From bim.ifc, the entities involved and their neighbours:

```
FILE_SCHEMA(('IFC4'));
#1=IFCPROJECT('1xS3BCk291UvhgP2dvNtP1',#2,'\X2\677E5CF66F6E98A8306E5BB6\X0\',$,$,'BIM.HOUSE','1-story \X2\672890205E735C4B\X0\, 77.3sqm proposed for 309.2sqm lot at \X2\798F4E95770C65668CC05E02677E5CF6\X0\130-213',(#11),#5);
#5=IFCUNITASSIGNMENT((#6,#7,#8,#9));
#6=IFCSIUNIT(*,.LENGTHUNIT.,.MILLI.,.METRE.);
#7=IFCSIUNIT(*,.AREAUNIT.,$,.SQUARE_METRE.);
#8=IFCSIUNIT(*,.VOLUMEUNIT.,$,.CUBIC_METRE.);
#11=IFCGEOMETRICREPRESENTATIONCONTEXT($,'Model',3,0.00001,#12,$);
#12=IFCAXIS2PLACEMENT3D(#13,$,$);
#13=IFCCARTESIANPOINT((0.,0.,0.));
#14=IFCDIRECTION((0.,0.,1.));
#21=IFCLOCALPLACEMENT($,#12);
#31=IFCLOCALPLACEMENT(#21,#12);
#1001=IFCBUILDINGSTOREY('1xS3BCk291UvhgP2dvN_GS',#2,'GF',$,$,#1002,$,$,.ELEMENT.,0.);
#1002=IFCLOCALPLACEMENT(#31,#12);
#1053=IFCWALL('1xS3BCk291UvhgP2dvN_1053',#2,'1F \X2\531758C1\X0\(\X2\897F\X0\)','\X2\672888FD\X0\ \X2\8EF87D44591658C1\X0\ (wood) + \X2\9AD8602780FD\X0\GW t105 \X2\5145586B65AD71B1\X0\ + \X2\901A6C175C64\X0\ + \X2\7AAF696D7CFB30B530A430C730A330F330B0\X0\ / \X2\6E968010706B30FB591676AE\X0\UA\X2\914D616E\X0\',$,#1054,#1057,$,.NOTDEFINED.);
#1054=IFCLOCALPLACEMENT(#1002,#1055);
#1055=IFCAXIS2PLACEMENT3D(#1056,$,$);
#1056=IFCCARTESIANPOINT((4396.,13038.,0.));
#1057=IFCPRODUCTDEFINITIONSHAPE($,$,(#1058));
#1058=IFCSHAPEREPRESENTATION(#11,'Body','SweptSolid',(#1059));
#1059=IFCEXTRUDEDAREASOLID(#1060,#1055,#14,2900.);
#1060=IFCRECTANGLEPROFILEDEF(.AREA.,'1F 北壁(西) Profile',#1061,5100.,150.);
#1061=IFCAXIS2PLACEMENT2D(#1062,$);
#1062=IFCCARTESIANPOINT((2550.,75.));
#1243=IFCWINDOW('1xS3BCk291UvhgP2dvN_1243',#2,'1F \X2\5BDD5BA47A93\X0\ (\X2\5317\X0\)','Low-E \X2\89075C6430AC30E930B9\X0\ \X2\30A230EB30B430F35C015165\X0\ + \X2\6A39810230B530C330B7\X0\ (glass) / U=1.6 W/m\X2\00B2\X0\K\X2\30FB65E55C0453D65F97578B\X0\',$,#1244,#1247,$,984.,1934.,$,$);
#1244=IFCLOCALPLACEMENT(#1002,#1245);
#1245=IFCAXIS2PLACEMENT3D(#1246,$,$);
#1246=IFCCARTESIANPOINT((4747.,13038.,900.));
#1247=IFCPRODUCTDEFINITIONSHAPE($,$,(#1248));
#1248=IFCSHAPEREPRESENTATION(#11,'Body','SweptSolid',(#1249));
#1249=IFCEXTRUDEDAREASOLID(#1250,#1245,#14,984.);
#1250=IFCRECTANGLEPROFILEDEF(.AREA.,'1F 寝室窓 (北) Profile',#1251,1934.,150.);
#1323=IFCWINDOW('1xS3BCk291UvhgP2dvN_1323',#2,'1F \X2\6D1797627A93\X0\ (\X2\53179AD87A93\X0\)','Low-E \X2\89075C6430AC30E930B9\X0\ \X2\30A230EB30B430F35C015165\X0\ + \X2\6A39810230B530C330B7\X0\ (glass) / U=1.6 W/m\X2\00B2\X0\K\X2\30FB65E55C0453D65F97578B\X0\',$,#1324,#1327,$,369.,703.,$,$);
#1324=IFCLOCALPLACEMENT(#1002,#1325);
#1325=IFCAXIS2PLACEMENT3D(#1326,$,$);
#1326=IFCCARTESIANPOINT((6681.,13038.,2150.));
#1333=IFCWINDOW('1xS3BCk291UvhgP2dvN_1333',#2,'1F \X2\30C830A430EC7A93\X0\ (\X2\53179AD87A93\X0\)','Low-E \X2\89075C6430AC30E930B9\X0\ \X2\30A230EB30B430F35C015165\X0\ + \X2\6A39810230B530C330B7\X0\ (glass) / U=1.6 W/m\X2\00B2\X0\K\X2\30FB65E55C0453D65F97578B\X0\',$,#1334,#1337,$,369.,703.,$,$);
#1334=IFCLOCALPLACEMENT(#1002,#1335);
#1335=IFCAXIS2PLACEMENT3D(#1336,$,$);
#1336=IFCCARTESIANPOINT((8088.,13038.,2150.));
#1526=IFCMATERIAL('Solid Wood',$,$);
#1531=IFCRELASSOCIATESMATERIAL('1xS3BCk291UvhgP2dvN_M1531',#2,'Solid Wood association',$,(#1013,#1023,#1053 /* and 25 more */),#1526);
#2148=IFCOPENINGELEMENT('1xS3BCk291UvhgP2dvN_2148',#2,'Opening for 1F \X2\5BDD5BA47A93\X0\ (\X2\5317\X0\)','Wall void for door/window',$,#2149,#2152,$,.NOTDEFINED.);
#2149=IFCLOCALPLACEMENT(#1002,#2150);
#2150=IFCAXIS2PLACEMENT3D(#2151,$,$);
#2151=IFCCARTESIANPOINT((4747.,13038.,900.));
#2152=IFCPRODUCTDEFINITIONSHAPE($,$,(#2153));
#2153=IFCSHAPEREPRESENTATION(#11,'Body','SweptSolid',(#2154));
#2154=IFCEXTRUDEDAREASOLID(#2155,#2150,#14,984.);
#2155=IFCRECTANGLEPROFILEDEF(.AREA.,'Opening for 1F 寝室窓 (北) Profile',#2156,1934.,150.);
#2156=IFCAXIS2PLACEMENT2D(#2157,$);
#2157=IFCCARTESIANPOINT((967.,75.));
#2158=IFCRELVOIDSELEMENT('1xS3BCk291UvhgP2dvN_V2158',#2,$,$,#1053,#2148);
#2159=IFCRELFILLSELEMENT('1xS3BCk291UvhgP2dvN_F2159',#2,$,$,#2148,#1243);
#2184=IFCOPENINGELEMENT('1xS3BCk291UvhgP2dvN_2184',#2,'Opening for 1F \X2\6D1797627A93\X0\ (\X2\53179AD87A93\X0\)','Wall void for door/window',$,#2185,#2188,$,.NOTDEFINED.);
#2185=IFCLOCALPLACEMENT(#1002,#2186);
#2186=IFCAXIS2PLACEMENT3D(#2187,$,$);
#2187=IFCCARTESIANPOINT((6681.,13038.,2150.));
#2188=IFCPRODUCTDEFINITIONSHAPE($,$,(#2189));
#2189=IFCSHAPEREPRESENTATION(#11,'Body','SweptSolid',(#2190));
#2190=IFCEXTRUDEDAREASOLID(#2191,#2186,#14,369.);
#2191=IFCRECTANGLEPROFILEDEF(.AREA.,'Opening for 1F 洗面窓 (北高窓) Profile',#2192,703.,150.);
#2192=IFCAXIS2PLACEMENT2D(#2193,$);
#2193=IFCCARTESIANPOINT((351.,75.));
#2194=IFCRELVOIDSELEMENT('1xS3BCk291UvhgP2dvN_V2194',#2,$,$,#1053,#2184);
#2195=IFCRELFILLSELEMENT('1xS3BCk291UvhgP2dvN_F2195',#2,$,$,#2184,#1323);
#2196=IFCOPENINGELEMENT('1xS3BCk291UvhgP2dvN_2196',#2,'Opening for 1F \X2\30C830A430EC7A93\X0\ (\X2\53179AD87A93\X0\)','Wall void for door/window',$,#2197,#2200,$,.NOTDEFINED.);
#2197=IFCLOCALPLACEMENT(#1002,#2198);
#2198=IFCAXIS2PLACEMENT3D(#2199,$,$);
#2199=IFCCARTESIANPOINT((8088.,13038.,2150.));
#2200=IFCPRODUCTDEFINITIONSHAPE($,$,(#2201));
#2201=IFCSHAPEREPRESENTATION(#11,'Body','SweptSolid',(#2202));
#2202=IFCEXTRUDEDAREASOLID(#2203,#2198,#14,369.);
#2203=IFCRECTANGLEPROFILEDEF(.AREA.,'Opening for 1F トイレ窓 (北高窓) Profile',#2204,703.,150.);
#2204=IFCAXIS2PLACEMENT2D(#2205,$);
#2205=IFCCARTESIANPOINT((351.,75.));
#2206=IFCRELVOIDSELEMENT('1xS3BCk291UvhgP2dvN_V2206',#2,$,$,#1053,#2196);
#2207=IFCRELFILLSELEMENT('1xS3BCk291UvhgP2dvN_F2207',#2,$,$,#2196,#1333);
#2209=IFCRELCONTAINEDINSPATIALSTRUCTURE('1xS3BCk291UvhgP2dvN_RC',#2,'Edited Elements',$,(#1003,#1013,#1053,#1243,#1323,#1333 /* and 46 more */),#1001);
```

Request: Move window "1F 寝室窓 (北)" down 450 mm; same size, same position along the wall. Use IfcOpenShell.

```python
import numpy as np
import ifcopenshell
import ifcopenshell.api.geometry
import ifcopenshell.util.placement
import ifcopenshell.util.unit

model = ifcopenshell.open("bim.ifc")
unit_scale = ifcopenshell.util.unit.calculate_unit_scale(model)

window = model.by_guid("1xS3BCk291UvhgP2dvN_1243")
opening = window.FillsVoids[0].RelatingOpeningElement
dz = -0.45 / unit_scale

shift = np.array([0.0, 0.0, dz])
# The window is not placed relative to its opening, so move both.
for product in (opening, window):
    matrix = ifcopenshell.util.placement.get_local_placement(product.ObjectPlacement)
    matrix[:3, 3] += shift
    ifcopenshell.api.geometry.edit_object_placement(model, product=product, matrix=matrix, is_si=False)

print(f"moved by {dz * unit_scale:+.3f} m")

model.write("bim_rev.ifc")
```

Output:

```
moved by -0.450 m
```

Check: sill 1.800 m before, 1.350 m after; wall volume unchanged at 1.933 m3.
